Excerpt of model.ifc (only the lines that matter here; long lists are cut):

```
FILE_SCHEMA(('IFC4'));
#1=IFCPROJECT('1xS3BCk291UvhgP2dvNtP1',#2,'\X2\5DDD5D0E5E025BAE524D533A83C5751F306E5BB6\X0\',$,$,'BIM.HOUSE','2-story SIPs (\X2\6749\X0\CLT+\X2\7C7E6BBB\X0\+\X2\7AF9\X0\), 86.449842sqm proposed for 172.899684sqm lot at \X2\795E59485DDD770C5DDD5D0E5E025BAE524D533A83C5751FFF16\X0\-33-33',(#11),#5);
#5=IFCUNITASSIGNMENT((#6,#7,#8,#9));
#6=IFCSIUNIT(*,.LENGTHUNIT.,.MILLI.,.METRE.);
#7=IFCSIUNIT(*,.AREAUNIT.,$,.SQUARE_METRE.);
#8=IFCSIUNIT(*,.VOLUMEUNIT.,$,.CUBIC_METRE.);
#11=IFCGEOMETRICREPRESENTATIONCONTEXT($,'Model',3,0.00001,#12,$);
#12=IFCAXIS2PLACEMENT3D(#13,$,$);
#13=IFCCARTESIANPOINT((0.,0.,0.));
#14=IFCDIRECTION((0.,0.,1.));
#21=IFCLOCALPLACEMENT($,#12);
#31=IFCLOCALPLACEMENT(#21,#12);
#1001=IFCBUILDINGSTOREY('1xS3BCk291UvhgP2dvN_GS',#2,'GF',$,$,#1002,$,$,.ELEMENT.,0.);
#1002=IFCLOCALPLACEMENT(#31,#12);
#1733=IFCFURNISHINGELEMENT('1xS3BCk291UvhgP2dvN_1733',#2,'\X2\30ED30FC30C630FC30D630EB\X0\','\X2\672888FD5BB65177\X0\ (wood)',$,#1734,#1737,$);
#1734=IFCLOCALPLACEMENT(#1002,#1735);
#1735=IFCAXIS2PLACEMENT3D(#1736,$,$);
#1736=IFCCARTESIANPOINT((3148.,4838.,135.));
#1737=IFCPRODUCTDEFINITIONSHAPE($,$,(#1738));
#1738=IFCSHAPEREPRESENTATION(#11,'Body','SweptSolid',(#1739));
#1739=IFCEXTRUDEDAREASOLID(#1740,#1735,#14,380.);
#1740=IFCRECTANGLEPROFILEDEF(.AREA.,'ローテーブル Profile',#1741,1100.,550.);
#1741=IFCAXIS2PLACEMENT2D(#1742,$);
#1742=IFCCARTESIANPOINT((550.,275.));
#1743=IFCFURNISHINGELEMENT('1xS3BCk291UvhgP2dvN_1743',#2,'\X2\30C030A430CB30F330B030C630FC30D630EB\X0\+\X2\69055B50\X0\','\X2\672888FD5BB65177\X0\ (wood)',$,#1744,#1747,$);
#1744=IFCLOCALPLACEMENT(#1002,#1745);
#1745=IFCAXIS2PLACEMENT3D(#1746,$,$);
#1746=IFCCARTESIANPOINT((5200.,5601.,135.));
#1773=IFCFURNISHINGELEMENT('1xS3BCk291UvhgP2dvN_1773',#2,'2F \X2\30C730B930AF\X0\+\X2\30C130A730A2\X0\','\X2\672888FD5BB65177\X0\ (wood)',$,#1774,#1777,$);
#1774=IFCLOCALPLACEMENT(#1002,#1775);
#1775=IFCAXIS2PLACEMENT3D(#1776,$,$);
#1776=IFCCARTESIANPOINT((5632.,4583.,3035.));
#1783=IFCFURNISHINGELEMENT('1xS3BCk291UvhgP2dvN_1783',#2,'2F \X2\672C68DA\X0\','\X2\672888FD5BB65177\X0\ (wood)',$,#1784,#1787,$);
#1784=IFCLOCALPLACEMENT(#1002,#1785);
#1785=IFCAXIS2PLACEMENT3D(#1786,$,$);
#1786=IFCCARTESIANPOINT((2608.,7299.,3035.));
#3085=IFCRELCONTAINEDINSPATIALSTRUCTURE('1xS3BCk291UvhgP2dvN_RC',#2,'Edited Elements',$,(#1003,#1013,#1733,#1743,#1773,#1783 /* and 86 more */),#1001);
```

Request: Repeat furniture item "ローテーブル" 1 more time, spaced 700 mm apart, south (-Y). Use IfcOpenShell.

```python
import numpy as np
import ifcopenshell
import ifcopenshell.api.geometry
import ifcopenshell.api.root
import ifcopenshell.util.element
import ifcopenshell.util.placement
import ifcopenshell.util.unit

model = ifcopenshell.open("model.ifc")
unit_scale = ifcopenshell.util.unit.calculate_unit_scale(model)


def reuse_history(source, copy):
    """copy_class also copies each property set's owner history, people and application; keep the originals."""
    for rel in copy.IsDefinedBy:
        if rel.is_a("IfcRelDefinesByProperties") and (history := rel.RelatingPropertyDefinition.OwnerHistory):
            rel.RelatingPropertyDefinition.OwnerHistory = source.OwnerHistory
            ifcopenshell.util.element.remove_deep2(model, history)


source = model.by_guid("1xS3BCk291UvhgP2dvN_1733")
base = ifcopenshell.util.placement.get_local_placement(source.ObjectPlacement)
step = np.array([0.0, -1.0, 0.0]) * 0.7 / unit_scale

for i in range(1, 2):
    copy = ifcopenshell.api.root.copy_class(model, product=source)
    copy.Representation = ifcopenshell.util.element.copy_deep(
        model, source.Representation, exclude=["IfcGeometricRepresentationContext", "IfcRepresentationMap"]
    )
    reuse_history(source, copy)
    matrix = base.copy()
    matrix[:3, 3] += i * step
    print("added at", matrix[:3, 3].round(3) + 0.0)
    ifcopenshell.api.geometry.edit_object_placement(model, product=copy, matrix=matrix, is_si=False)

model.write("model_v2.ifc")
```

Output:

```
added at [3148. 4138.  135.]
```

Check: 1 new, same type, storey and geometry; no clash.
